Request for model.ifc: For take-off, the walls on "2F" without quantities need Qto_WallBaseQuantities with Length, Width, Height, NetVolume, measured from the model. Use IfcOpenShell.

First a look at what the model holds.

```python
import ifcopenshell
import ifcopenshell.util.element
import ifcopenshell.util.unit

model = ifcopenshell.open("model.ifc")
print(model.schema)
for unit_type in ("LENGTHUNIT", "AREAUNIT", "VOLUMEUNIT"):
    print(unit_type, ifcopenshell.util.unit.calculate_unit_scale(model, unit_type))
storey = next(s for s in model.by_type("IfcBuildingStorey") if s.Name == "2F")
walls = [e for e in ifcopenshell.util.element.get_decomposition(storey) if e.is_a("IfcWall")]
for e in sorted(walls, key=lambda e: e.id()):
    print(e.id(), e.is_a(), e.Name, list(ifcopenshell.util.element.get_psets(e, qtos_only=True)), sep=" | ")
```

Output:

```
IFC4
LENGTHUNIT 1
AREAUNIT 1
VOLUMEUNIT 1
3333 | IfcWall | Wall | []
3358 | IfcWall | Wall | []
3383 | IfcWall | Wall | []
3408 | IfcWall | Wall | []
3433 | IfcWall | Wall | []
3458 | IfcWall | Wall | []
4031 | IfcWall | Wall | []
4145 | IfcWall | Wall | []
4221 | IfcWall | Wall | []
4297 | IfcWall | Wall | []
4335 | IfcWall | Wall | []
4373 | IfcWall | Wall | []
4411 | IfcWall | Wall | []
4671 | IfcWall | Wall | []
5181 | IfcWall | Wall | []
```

```python
import ifcopenshell
import ifcopenshell.api.pset
import ifcopenshell.geom
import ifcopenshell.util.element
import ifcopenshell.util.shape
import ifcopenshell.util.unit

model = ifcopenshell.open("model.ifc")
unit_scale = ifcopenshell.util.unit.calculate_unit_scale(model)
volume_scale = ifcopenshell.util.unit.calculate_unit_scale(model, "VOLUMEUNIT")
settings = ifcopenshell.geom.settings()

storey = next(s for s in model.by_type("IfcBuildingStorey") if s.Name == "2F")
walls = [e for e in ifcopenshell.util.element.get_decomposition(storey) if e.is_a("IfcWall")]

for e in sorted(walls, key=lambda e: e.id()):
    if ifcopenshell.util.element.get_psets(e, qtos_only=True, should_inherit=False):
        continue
    # Geometry comes back in metres, in the element's own axes.
    shape = ifcopenshell.geom.create_shape(settings, e)
    values = {
        "Length": ifcopenshell.util.shape.get_x(shape.geometry) / unit_scale,
        "Width": ifcopenshell.util.shape.get_y(shape.geometry) / unit_scale,
        "Height": ifcopenshell.util.shape.get_z(shape.geometry) / unit_scale,
        "NetVolume": ifcopenshell.util.shape.get_volume(shape.geometry) / volume_scale,
    }
    qto = ifcopenshell.api.pset.add_qto(model, product=e, name="Qto_WallBaseQuantities")
    ifcopenshell.api.pset.edit_qto(model, qto=qto, properties=values)
    print(e.id(), {k: round(v, 3) for k, v in values.items()})

model.write("model_updated.ifc")
```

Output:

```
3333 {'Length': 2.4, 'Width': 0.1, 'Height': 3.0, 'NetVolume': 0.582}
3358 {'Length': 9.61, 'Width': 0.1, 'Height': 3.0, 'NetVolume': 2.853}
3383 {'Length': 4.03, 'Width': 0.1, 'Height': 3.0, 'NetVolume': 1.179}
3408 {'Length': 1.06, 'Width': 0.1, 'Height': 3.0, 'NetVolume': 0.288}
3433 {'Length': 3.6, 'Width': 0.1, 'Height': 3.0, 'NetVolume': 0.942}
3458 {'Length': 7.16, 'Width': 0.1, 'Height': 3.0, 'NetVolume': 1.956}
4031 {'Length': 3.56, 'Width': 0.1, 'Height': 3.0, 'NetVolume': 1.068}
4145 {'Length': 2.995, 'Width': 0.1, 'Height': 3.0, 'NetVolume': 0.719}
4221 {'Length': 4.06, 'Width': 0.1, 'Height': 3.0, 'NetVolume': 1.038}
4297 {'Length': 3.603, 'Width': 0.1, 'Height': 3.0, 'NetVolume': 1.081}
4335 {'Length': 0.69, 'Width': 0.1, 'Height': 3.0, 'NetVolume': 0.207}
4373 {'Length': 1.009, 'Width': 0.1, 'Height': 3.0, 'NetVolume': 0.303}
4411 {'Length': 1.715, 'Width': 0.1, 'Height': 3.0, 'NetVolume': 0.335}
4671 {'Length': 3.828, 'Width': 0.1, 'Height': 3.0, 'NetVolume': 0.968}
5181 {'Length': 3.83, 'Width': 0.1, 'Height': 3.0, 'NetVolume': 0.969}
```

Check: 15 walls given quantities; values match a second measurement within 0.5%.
